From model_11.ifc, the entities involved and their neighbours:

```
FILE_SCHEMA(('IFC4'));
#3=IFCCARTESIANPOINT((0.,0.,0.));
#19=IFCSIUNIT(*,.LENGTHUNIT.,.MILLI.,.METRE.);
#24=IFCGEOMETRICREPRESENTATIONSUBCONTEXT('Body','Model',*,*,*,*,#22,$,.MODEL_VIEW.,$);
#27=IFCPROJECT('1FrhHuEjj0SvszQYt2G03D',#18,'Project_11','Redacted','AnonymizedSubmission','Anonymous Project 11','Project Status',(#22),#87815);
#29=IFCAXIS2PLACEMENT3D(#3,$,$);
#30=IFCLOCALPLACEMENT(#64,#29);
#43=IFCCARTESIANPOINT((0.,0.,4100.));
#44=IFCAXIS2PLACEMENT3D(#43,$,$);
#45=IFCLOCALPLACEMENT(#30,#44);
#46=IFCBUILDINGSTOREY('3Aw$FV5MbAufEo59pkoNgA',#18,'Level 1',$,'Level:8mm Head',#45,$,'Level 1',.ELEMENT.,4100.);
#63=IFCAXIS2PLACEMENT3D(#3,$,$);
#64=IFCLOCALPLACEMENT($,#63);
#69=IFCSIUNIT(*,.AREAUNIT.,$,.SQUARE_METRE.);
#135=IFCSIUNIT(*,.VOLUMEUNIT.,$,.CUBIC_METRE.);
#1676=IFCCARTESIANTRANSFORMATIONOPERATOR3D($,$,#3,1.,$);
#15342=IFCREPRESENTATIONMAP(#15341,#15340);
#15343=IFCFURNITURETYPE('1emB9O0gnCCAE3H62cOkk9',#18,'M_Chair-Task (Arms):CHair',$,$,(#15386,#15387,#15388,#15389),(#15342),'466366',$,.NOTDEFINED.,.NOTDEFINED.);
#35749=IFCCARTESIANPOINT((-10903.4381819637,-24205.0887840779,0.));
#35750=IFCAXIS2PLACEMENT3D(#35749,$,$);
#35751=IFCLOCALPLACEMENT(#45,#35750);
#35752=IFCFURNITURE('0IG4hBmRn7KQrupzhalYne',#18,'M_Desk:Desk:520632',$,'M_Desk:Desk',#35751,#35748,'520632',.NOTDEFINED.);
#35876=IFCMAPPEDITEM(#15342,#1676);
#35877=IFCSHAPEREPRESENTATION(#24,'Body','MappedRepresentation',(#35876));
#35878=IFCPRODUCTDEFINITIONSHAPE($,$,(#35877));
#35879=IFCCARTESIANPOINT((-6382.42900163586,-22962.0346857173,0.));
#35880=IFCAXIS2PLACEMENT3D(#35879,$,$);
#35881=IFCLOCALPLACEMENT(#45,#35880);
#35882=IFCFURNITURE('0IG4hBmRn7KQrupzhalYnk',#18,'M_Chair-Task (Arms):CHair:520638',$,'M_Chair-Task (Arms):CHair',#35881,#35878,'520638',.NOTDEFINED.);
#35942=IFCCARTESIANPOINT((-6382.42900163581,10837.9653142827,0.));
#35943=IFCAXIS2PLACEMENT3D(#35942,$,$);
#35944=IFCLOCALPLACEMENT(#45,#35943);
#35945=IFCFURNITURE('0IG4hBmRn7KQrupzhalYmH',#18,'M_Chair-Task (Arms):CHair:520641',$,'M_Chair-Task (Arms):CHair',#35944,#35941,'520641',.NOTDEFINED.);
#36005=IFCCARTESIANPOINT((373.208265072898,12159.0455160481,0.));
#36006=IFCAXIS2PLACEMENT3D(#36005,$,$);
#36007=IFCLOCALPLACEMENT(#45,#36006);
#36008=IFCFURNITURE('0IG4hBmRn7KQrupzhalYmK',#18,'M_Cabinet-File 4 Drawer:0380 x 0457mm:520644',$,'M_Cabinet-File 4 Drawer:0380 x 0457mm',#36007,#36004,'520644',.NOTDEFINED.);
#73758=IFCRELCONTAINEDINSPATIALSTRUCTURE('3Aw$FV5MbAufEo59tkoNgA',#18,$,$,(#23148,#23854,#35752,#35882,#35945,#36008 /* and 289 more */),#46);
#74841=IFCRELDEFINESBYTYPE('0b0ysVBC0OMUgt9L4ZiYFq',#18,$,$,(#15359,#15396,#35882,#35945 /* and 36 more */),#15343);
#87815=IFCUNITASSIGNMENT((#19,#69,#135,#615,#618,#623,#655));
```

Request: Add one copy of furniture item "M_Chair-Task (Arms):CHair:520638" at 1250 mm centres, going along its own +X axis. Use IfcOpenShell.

```python
import ifcopenshell
import ifcopenshell.api.geometry
import ifcopenshell.api.root
import ifcopenshell.util.element
import ifcopenshell.util.placement

model = ifcopenshell.open("model_11.ifc")


def reuse_history(source, copy):
    """copy_class also copies each property set's owner history, people and application; keep the originals."""
    for rel in copy.IsDefinedBy:
        if rel.is_a("IfcRelDefinesByProperties") and (history := rel.RelatingPropertyDefinition.OwnerHistory):
            rel.RelatingPropertyDefinition.OwnerHistory = source.OwnerHistory
            ifcopenshell.util.element.remove_deep2(model, history)


source = model.by_guid("0IG4hBmRn7KQrupzhalYnk")
base = ifcopenshell.util.placement.get_local_placement(source.ObjectPlacement)
step = base[:3, 0] * 1250.0

for i in range(1, 2):
    copy = ifcopenshell.api.root.copy_class(model, product=source)
    copy.Representation = ifcopenshell.util.element.copy_deep(
        model, source.Representation, exclude=["IfcGeometricRepresentationContext", "IfcRepresentationMap"]
    )
    copy.Name = "M_Chair-Task (Arms):CHair"
    copy.Tag = None
    reuse_history(source, copy)
    matrix = base.copy()
    matrix[:3, 3] += i * step
    print("added at", matrix[:3, 3].round(3) + 0.0)
    ifcopenshell.api.geometry.edit_object_placement(model, product=copy, matrix=matrix, is_si=False)

model.write("model_11-out.ifc")
```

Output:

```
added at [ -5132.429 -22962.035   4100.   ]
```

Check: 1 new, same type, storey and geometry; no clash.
